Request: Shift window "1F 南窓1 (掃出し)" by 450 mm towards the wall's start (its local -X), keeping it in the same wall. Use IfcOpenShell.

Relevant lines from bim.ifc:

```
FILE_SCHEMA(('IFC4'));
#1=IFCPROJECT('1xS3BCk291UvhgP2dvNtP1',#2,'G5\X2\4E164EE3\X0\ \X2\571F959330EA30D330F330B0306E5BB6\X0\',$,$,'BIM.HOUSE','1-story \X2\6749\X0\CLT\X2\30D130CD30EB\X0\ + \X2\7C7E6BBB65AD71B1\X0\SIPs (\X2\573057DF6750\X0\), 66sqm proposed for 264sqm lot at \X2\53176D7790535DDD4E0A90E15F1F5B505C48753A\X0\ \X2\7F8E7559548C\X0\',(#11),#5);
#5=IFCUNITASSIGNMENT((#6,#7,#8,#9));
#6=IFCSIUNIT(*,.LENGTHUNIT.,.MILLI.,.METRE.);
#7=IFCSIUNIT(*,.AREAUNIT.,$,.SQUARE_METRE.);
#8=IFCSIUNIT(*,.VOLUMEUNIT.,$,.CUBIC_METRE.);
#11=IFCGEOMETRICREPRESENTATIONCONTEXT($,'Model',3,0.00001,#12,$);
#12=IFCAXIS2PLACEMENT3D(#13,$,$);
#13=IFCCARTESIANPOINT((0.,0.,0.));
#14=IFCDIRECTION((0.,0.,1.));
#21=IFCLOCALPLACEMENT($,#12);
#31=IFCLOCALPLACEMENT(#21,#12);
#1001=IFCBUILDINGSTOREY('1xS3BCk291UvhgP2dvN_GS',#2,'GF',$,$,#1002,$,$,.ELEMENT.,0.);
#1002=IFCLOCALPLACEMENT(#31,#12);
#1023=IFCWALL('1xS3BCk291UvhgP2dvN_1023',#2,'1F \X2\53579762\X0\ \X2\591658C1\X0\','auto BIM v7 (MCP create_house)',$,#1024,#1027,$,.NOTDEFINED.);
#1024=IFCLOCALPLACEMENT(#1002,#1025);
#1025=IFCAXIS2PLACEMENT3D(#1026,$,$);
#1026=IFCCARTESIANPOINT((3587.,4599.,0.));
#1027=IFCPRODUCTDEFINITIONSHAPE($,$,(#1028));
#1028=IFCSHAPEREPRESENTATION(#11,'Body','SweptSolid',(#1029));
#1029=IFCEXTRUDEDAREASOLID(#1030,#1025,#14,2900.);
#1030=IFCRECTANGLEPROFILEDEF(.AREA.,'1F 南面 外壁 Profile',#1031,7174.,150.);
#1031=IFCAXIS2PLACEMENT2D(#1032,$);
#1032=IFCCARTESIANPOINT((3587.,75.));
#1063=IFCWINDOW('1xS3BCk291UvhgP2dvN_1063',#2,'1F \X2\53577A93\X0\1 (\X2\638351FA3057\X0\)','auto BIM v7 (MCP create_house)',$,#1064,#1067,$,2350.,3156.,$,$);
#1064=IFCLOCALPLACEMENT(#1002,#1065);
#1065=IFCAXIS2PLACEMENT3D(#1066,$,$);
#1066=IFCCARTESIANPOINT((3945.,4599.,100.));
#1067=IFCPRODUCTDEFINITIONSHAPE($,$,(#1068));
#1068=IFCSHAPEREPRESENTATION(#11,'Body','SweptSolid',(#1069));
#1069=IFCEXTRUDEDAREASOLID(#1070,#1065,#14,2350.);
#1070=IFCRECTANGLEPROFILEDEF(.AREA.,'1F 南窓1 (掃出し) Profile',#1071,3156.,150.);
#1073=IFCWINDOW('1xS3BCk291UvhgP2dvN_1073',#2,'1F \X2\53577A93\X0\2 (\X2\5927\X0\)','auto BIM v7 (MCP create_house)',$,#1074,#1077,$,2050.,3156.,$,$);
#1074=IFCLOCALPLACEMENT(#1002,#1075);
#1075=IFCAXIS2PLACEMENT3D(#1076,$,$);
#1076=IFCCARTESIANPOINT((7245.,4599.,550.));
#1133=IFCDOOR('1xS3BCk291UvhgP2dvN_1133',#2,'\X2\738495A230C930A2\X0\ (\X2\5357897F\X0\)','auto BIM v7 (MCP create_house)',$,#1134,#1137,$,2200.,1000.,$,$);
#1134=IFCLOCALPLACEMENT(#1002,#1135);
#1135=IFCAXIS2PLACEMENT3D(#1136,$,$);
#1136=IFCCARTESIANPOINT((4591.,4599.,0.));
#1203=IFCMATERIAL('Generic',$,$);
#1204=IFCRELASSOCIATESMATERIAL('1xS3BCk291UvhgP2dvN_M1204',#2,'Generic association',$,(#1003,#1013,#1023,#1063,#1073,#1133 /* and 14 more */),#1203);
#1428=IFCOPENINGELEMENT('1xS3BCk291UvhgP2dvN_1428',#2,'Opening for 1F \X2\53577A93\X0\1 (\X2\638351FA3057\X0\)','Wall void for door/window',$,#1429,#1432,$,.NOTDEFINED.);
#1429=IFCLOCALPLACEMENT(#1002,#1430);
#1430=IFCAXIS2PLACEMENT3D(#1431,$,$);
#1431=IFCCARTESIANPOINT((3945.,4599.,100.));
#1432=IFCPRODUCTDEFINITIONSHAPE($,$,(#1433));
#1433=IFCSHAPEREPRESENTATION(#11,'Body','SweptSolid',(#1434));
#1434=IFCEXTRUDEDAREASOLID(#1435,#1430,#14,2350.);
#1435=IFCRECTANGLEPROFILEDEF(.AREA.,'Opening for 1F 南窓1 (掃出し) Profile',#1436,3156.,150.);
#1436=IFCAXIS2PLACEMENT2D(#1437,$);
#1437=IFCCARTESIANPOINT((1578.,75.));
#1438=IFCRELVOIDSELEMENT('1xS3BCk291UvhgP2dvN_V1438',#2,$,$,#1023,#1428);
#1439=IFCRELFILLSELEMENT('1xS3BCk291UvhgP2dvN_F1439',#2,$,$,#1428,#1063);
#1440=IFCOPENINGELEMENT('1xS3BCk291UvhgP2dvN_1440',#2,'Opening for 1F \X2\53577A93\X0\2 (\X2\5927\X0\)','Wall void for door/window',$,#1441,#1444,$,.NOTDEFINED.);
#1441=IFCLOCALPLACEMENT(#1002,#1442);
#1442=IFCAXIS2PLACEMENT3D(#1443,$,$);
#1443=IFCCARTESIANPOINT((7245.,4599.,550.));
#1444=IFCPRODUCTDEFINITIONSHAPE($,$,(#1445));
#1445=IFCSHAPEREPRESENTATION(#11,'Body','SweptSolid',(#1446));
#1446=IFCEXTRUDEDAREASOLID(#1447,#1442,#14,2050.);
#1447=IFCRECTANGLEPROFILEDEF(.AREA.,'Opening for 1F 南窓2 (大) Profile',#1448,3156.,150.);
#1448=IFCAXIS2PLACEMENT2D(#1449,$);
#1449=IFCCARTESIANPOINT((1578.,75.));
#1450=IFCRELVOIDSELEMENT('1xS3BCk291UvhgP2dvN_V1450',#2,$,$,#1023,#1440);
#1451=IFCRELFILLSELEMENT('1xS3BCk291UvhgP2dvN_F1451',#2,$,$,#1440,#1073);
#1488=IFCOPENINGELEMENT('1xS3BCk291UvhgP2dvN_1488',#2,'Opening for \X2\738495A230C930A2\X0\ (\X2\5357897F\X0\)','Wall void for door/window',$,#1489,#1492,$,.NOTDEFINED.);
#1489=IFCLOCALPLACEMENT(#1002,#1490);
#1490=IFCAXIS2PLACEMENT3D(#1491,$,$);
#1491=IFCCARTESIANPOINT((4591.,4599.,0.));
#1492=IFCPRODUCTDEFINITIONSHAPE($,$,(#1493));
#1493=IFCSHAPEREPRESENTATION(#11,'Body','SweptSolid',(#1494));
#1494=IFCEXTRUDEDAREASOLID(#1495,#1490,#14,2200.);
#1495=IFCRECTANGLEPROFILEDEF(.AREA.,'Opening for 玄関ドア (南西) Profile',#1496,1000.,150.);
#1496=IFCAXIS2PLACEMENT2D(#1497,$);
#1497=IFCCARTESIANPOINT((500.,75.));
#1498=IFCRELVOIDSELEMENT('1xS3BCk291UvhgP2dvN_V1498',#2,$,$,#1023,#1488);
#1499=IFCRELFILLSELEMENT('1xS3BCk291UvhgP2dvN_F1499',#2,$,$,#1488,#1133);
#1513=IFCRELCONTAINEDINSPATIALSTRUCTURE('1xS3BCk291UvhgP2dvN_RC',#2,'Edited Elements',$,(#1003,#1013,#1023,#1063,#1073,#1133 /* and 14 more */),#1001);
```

```python
import ifcopenshell
import ifcopenshell.api.geometry
import ifcopenshell.util.placement

model = ifcopenshell.open("bim.ifc")

window = model.by_guid("1xS3BCk291UvhgP2dvN_1063")
opening = window.FillsVoids[0].RelatingOpeningElement
wall = opening.VoidsElements[0].RelatingBuildingElement

wall_matrix = ifcopenshell.util.placement.get_local_placement(wall.ObjectPlacement)
shift = wall_matrix[:3, 0] * -450.0
before = ifcopenshell.util.placement.get_local_placement(window.ObjectPlacement)[:3, 3].copy()

# The window is not placed relative to its opening, so move both.
for product in (opening, window):
    matrix = ifcopenshell.util.placement.get_local_placement(product.ObjectPlacement)
    matrix[:3, 3] += shift
    ifcopenshell.api.geometry.edit_object_placement(model, product=product, matrix=matrix, is_si=False)

after = ifcopenshell.util.placement.get_local_placement(window.ObjectPlacement)[:3, 3]
print("window moved by", (after - before).round(3) + 0.0)

model.write("bim_edited.ifc")
```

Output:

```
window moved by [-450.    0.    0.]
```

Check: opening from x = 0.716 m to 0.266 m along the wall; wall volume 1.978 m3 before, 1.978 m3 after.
